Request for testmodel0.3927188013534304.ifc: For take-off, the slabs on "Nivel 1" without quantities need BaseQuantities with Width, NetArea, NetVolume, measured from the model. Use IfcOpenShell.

First a look at what the model holds.

```python
import ifcopenshell
import ifcopenshell.util.element
import ifcopenshell.util.unit

model = ifcopenshell.open("testmodel0.3927188013534304.ifc")
print(model.schema)
for unit_type in ("LENGTHUNIT", "AREAUNIT", "VOLUMEUNIT"):
    print(unit_type, ifcopenshell.util.unit.calculate_unit_scale(model, unit_type))
storey = next(s for s in model.by_type("IfcBuildingStorey") if s.Name == "Nivel 1")
slabs = [e for e in ifcopenshell.util.element.get_decomposition(storey) if e.is_a("IfcSlab")]
for e in sorted(slabs, key=lambda e: e.id()):
    print(e.id(), e.is_a(), e.Name, list(ifcopenshell.util.element.get_psets(e, qtos_only=True)), sep=" | ")
```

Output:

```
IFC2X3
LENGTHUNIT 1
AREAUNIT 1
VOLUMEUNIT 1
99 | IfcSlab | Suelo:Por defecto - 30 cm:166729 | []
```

```python
import ifcopenshell
import ifcopenshell.api.pset
import ifcopenshell.geom
import ifcopenshell.util.element
import ifcopenshell.util.shape
import ifcopenshell.util.unit

model = ifcopenshell.open("testmodel0.3927188013534304.ifc")
unit_scale = ifcopenshell.util.unit.calculate_unit_scale(model)
area_scale = ifcopenshell.util.unit.calculate_unit_scale(model, "AREAUNIT")
volume_scale = ifcopenshell.util.unit.calculate_unit_scale(model, "VOLUMEUNIT")
settings = ifcopenshell.geom.settings()

storey = next(s for s in model.by_type("IfcBuildingStorey") if s.Name == "Nivel 1")
slabs = [e for e in ifcopenshell.util.element.get_decomposition(storey) if e.is_a("IfcSlab")]

for e in sorted(slabs, key=lambda e: e.id()):
    if ifcopenshell.util.element.get_psets(e, qtos_only=True, should_inherit=False):
        continue
    # Geometry comes back in metres, in the element's own axes.
    shape = ifcopenshell.geom.create_shape(settings, e)
    values = {
        "Width": ifcopenshell.util.shape.get_z(shape.geometry) / unit_scale,
        "NetArea": ifcopenshell.util.shape.get_footprint_area(shape.geometry) / area_scale,
        "NetVolume": ifcopenshell.util.shape.get_volume(shape.geometry) / volume_scale,
    }
    qto = ifcopenshell.api.pset.add_qto(model, product=e, name="BaseQuantities")
    ifcopenshell.api.pset.edit_qto(model, qto=qto, properties=values)
    print(e.id(), {k: round(v, 3) for k, v in values.items()})

model.write("testmodel0.3927188013534304-out.ifc")
```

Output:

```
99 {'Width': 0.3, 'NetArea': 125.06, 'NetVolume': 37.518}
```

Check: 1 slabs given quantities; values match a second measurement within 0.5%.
